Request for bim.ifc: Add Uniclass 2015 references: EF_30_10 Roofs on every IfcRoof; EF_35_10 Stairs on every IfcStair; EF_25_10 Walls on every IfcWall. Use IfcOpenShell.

First a look at what the model holds.

```python
import ifcopenshell

model = ifcopenshell.open("bim.ifc")
print(model.schema)
print("classifications:", [c.Name for c in model.by_type("IfcClassification")])
for ifc_class in ("IfcDoor", "IfcRoof", "IfcStair", "IfcWall", "IfcWindow"):
    print(ifc_class, len(model.by_type(ifc_class)))
```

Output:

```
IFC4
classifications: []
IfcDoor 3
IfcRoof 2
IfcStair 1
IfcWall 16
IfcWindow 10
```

```python
import ifcopenshell
import ifcopenshell.api.classification

model = ifcopenshell.open("bim.ifc")

system = ifcopenshell.api.classification.add_classification(model, classification="Uniclass 2015")

codes = {
    "IfcRoof": ("EF_30_10", "Roofs"),
    "IfcStair": ("EF_35_10", "Stairs"),
    "IfcWall": ("EF_25_10", "Walls"),
}
for ifc_class, (code, name) in codes.items():
    products = model.by_type(ifc_class)
    ifcopenshell.api.classification.add_reference(
        model, products=products, classification=system, identification=code, name=name
    )
    print(code, len(products))

model.write("bim_v2.ifc")
```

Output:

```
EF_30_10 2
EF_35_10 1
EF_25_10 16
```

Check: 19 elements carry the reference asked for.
